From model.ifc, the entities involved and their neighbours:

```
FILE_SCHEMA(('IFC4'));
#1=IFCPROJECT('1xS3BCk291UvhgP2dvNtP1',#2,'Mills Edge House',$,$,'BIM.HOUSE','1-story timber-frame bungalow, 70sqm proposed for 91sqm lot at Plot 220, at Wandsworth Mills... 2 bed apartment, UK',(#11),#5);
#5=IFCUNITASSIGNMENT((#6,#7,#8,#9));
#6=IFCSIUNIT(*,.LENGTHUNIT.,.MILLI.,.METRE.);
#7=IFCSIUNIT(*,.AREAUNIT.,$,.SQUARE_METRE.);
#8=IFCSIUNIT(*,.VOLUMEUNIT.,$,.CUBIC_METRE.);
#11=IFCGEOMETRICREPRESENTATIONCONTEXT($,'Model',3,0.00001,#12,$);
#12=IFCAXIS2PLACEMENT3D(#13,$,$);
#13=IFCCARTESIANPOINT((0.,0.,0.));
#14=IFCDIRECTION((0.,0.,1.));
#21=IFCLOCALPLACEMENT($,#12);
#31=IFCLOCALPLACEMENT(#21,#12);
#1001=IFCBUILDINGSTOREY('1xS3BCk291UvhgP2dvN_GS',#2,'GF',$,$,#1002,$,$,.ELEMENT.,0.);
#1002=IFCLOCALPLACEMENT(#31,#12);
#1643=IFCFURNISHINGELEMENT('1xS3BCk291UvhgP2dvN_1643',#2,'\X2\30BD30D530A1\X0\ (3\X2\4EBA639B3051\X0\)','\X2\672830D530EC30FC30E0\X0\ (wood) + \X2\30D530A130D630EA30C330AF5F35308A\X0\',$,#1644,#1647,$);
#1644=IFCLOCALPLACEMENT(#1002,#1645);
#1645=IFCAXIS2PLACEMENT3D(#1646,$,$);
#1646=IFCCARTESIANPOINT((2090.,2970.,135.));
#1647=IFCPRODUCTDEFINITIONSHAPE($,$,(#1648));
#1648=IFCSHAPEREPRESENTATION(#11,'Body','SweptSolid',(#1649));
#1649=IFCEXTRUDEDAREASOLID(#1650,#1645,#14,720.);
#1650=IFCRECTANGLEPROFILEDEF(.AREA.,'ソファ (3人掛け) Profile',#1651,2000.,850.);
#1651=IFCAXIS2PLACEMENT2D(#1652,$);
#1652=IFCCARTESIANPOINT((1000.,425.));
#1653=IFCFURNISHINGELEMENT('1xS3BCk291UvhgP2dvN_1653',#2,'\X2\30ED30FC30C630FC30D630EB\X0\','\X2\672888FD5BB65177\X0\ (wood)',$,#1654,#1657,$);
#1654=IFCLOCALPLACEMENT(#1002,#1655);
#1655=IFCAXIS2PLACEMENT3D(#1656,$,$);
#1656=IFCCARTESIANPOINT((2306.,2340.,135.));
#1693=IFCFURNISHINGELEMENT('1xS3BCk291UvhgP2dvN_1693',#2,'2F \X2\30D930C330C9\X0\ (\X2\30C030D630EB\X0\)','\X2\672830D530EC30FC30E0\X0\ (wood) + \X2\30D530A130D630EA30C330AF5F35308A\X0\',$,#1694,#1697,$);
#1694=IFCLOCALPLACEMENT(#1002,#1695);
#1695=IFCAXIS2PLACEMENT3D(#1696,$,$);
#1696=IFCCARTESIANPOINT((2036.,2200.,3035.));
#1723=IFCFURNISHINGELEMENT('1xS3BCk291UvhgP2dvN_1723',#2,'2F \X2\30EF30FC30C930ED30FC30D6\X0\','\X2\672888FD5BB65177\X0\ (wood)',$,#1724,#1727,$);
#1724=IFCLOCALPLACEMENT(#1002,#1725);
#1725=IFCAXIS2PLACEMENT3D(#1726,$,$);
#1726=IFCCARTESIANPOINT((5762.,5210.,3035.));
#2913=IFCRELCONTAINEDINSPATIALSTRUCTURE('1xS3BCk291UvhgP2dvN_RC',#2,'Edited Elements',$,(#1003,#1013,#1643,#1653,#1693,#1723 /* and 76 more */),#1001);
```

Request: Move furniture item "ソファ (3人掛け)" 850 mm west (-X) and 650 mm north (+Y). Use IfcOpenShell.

```python
import ifcopenshell
import ifcopenshell.api.geometry
import ifcopenshell.util.placement

model = ifcopenshell.open("model.ifc")

item = model.by_guid("1xS3BCk291UvhgP2dvN_1643")
matrix = ifcopenshell.util.placement.get_local_placement(item.ObjectPlacement)
matrix[0, 3] -= 850.0
matrix[1, 3] += 650.0
ifcopenshell.api.geometry.edit_object_placement(model, product=item, matrix=matrix, is_si=False)

print(ifcopenshell.util.placement.get_local_placement(item.ObjectPlacement).round(3) + 0.0)

model.write("model-out.ifc")
```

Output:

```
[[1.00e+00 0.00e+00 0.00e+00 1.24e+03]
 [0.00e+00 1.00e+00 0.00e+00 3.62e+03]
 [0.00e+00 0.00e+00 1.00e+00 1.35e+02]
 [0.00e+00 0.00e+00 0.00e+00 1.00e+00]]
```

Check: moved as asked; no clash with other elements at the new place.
